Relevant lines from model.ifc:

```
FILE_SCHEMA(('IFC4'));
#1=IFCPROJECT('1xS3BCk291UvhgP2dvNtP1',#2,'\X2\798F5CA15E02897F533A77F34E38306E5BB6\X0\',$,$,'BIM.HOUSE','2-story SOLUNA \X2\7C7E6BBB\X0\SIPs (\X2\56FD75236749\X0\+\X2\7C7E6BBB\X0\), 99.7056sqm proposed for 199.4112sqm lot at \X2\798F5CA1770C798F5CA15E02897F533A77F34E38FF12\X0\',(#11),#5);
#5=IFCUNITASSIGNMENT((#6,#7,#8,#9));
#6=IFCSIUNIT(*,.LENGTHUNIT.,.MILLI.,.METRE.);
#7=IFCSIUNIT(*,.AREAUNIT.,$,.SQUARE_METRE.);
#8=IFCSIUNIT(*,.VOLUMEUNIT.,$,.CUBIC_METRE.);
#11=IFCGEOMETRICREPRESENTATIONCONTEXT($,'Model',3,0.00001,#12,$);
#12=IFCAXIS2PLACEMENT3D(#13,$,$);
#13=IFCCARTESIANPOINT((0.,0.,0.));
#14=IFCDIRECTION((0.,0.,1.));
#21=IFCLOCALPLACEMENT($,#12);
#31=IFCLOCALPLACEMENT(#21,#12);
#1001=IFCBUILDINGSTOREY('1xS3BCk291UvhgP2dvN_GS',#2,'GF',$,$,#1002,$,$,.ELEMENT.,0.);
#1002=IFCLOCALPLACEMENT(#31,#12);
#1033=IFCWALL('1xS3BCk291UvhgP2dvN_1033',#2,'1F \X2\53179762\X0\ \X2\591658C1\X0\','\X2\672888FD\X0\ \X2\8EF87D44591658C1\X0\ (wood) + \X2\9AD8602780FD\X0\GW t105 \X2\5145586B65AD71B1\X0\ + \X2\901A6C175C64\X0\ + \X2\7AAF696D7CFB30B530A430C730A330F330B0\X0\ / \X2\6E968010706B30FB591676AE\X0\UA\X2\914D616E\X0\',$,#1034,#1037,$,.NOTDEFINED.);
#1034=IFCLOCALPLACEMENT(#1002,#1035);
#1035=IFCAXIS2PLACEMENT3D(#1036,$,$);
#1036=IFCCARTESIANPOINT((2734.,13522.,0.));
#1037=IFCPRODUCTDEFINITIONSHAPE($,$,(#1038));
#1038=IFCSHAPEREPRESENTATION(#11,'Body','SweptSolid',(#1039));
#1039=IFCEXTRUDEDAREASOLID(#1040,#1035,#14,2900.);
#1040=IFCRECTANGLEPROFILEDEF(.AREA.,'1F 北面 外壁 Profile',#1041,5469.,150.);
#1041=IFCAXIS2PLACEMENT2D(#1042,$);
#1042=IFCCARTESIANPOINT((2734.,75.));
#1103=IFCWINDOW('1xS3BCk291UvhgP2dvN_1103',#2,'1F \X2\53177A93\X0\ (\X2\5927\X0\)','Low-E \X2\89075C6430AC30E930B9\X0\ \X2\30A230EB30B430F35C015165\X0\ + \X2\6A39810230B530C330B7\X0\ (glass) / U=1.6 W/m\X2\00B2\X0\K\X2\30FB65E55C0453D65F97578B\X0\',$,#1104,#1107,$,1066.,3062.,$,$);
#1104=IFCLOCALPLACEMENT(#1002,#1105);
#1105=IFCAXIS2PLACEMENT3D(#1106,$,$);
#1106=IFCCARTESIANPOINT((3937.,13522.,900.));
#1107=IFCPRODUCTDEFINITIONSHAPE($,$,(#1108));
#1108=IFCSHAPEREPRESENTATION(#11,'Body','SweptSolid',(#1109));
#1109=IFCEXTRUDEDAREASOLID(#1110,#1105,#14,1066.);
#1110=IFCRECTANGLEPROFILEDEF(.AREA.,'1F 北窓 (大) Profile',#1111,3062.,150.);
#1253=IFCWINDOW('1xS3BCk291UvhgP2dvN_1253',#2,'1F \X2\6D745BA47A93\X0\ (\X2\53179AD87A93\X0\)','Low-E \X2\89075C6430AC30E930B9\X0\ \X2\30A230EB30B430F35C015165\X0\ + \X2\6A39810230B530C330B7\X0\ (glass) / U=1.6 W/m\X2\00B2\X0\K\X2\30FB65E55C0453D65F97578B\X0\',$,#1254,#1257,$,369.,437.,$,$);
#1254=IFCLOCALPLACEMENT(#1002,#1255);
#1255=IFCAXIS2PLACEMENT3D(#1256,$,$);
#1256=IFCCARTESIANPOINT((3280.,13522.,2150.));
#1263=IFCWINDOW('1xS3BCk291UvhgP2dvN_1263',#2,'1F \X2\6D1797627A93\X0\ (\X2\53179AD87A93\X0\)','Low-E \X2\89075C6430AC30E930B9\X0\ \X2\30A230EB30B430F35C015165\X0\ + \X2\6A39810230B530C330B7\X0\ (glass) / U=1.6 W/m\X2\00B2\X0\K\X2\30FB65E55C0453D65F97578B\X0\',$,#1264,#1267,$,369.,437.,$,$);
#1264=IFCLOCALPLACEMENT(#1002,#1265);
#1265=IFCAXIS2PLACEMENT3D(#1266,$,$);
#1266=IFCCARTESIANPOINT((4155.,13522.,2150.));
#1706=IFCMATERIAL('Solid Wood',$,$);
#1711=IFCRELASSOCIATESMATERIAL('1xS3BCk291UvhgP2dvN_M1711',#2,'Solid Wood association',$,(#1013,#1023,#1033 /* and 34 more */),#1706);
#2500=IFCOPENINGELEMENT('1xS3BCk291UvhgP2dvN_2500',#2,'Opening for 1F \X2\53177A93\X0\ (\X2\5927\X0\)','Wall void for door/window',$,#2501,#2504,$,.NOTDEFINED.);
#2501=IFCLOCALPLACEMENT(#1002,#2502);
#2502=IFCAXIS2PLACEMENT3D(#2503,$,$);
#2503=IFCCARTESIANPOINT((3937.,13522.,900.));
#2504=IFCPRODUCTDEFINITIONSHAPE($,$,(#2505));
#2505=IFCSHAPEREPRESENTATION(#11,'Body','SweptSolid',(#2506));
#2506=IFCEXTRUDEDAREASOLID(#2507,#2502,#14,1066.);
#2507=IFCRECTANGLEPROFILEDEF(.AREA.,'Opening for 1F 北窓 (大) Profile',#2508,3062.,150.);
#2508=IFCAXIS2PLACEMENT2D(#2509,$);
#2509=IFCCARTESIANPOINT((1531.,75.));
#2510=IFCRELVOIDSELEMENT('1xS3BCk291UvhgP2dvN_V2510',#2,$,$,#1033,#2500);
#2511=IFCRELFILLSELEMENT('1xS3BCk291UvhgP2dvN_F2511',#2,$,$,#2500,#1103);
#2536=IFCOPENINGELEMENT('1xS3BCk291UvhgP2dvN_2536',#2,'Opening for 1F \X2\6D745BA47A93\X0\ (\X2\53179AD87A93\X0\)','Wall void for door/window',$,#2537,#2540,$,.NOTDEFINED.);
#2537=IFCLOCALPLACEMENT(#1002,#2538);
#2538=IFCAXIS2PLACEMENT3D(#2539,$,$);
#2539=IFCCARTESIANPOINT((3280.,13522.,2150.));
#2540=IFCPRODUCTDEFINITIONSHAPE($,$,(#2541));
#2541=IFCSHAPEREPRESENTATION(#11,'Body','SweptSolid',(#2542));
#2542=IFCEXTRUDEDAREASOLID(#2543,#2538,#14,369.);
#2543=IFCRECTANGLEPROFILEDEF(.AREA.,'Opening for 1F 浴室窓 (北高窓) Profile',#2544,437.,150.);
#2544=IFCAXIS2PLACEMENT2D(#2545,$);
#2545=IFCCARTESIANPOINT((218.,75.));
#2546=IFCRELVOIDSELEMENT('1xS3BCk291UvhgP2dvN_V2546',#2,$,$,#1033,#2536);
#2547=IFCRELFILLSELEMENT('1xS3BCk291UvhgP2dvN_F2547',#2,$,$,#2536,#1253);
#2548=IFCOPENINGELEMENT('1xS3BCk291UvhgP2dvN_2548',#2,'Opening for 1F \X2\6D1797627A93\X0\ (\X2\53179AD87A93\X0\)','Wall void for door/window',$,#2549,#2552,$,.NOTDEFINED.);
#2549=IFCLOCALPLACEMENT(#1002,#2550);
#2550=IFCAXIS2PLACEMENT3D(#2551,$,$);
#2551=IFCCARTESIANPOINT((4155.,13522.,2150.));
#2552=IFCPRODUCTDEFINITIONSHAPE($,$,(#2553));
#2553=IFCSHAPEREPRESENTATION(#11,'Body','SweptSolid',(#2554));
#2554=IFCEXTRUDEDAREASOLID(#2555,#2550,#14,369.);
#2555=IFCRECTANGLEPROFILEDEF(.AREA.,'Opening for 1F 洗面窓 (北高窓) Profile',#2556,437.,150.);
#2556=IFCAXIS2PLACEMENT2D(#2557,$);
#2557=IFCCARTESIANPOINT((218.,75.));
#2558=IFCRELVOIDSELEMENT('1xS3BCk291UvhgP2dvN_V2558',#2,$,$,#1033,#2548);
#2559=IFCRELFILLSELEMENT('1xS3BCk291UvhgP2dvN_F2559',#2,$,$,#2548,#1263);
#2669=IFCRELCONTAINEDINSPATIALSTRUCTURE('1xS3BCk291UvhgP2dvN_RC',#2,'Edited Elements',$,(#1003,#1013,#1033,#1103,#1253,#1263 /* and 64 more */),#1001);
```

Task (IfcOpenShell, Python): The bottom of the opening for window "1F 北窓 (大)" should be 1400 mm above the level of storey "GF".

```python
import numpy as np
import ifcopenshell
import ifcopenshell.api.geometry
import ifcopenshell.geom
import ifcopenshell.util.element
import ifcopenshell.util.placement
import ifcopenshell.util.shape
import ifcopenshell.util.unit

model = ifcopenshell.open("model.ifc")
unit_scale = ifcopenshell.util.unit.calculate_unit_scale(model)

window = model.by_guid("1xS3BCk291UvhgP2dvN_1103")
opening = window.FillsVoids[0].RelatingOpeningElement
storey = ifcopenshell.util.element.get_container(window, ifc_class="IfcBuildingStorey")
level = ifcopenshell.util.placement.get_local_placement(storey.ObjectPlacement)[2, 3]

# The opening's origin need not be at the sill, so measure its lowest point.
shape = ifcopenshell.geom.create_shape(ifcopenshell.geom.settings(), opening)
bottom = ifcopenshell.util.shape.get_shape_bottom_elevation(shape, shape.geometry) / unit_scale
dz = level + 1.4 / unit_scale - bottom

shift = np.array([0.0, 0.0, dz])
# The window is not placed relative to its opening, so move both.
for product in (opening, window):
    matrix = ifcopenshell.util.placement.get_local_placement(product.ObjectPlacement)
    matrix[:3, 3] += shift
    ifcopenshell.api.geometry.edit_object_placement(model, product=product, matrix=matrix, is_si=False)

print(f"moved by {dz * unit_scale:+.3f} m")

model.write("model_edited.ifc")
```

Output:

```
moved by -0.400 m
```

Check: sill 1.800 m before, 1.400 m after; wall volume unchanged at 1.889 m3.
